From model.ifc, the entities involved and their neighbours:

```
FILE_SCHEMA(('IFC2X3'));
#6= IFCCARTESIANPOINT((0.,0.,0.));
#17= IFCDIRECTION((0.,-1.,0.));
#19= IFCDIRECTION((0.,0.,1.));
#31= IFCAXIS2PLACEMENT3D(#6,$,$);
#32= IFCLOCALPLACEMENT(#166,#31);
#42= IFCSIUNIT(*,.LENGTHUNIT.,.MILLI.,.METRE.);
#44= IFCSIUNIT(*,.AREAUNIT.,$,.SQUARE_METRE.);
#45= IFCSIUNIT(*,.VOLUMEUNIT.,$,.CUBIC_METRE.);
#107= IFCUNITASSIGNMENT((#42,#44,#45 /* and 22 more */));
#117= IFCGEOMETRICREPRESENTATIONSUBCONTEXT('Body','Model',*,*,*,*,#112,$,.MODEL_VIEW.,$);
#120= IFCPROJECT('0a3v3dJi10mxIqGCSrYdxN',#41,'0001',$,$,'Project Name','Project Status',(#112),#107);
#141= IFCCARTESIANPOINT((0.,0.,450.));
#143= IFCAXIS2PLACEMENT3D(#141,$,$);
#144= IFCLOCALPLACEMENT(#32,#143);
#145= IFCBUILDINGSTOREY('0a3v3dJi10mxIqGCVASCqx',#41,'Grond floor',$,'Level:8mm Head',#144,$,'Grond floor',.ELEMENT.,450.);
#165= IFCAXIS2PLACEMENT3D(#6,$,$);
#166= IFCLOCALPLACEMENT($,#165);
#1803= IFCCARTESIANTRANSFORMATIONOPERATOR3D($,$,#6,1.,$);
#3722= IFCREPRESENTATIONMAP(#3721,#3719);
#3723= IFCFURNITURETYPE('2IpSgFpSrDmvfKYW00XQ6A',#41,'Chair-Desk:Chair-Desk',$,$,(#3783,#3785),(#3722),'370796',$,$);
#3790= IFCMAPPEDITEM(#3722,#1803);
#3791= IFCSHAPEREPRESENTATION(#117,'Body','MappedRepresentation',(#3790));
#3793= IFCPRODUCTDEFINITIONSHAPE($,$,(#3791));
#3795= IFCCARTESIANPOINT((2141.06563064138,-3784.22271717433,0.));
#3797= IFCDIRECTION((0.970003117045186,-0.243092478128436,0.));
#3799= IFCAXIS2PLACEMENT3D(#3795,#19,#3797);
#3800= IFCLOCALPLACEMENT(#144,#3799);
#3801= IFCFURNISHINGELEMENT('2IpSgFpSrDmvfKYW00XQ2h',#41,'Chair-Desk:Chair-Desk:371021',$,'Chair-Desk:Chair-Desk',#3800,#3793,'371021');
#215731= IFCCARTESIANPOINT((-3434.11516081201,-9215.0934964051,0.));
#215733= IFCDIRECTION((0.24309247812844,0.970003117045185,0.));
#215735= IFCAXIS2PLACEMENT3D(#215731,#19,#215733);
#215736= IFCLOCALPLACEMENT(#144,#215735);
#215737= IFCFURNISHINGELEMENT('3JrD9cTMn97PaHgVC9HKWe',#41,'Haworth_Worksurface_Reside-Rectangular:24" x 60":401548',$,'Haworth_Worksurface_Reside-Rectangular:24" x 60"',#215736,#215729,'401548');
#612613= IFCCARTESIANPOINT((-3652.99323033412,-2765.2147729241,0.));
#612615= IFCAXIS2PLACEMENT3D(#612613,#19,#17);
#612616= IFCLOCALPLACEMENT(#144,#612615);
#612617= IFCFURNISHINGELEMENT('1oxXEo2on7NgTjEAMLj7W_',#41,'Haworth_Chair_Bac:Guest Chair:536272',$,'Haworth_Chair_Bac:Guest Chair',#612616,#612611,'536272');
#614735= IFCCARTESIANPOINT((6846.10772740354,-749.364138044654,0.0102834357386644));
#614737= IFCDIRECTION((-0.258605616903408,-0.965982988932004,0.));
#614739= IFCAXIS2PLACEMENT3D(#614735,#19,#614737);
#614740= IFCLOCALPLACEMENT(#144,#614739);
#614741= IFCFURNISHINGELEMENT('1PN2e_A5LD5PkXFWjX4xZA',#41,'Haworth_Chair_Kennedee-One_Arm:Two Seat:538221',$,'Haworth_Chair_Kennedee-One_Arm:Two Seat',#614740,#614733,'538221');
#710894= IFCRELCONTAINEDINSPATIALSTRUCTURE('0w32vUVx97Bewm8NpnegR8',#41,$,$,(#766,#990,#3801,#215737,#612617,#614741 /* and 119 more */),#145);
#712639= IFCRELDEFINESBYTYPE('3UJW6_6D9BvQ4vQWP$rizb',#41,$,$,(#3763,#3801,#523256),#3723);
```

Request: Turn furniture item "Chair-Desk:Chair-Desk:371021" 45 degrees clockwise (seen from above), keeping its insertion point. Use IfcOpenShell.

```python
import ifcopenshell
import ifcopenshell.api.geometry
import ifcopenshell.util.placement

model = ifcopenshell.open("model.ifc")

item = model.by_id(3801)
matrix = ifcopenshell.util.placement.get_local_placement(item.ObjectPlacement)
matrix = matrix @ ifcopenshell.util.placement.rotation(-45, "Z")
ifcopenshell.api.geometry.edit_object_placement(model, product=item, matrix=matrix, is_si=False)

print(ifcopenshell.util.placement.get_local_placement(item.ObjectPlacement).round(3) + 0.0)

model.write("model_v2.ifc")
```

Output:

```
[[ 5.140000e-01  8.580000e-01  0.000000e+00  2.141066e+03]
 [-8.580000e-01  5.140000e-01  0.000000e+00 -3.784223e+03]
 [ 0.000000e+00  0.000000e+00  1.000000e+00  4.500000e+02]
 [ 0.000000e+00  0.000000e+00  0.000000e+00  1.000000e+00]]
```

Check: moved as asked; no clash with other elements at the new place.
